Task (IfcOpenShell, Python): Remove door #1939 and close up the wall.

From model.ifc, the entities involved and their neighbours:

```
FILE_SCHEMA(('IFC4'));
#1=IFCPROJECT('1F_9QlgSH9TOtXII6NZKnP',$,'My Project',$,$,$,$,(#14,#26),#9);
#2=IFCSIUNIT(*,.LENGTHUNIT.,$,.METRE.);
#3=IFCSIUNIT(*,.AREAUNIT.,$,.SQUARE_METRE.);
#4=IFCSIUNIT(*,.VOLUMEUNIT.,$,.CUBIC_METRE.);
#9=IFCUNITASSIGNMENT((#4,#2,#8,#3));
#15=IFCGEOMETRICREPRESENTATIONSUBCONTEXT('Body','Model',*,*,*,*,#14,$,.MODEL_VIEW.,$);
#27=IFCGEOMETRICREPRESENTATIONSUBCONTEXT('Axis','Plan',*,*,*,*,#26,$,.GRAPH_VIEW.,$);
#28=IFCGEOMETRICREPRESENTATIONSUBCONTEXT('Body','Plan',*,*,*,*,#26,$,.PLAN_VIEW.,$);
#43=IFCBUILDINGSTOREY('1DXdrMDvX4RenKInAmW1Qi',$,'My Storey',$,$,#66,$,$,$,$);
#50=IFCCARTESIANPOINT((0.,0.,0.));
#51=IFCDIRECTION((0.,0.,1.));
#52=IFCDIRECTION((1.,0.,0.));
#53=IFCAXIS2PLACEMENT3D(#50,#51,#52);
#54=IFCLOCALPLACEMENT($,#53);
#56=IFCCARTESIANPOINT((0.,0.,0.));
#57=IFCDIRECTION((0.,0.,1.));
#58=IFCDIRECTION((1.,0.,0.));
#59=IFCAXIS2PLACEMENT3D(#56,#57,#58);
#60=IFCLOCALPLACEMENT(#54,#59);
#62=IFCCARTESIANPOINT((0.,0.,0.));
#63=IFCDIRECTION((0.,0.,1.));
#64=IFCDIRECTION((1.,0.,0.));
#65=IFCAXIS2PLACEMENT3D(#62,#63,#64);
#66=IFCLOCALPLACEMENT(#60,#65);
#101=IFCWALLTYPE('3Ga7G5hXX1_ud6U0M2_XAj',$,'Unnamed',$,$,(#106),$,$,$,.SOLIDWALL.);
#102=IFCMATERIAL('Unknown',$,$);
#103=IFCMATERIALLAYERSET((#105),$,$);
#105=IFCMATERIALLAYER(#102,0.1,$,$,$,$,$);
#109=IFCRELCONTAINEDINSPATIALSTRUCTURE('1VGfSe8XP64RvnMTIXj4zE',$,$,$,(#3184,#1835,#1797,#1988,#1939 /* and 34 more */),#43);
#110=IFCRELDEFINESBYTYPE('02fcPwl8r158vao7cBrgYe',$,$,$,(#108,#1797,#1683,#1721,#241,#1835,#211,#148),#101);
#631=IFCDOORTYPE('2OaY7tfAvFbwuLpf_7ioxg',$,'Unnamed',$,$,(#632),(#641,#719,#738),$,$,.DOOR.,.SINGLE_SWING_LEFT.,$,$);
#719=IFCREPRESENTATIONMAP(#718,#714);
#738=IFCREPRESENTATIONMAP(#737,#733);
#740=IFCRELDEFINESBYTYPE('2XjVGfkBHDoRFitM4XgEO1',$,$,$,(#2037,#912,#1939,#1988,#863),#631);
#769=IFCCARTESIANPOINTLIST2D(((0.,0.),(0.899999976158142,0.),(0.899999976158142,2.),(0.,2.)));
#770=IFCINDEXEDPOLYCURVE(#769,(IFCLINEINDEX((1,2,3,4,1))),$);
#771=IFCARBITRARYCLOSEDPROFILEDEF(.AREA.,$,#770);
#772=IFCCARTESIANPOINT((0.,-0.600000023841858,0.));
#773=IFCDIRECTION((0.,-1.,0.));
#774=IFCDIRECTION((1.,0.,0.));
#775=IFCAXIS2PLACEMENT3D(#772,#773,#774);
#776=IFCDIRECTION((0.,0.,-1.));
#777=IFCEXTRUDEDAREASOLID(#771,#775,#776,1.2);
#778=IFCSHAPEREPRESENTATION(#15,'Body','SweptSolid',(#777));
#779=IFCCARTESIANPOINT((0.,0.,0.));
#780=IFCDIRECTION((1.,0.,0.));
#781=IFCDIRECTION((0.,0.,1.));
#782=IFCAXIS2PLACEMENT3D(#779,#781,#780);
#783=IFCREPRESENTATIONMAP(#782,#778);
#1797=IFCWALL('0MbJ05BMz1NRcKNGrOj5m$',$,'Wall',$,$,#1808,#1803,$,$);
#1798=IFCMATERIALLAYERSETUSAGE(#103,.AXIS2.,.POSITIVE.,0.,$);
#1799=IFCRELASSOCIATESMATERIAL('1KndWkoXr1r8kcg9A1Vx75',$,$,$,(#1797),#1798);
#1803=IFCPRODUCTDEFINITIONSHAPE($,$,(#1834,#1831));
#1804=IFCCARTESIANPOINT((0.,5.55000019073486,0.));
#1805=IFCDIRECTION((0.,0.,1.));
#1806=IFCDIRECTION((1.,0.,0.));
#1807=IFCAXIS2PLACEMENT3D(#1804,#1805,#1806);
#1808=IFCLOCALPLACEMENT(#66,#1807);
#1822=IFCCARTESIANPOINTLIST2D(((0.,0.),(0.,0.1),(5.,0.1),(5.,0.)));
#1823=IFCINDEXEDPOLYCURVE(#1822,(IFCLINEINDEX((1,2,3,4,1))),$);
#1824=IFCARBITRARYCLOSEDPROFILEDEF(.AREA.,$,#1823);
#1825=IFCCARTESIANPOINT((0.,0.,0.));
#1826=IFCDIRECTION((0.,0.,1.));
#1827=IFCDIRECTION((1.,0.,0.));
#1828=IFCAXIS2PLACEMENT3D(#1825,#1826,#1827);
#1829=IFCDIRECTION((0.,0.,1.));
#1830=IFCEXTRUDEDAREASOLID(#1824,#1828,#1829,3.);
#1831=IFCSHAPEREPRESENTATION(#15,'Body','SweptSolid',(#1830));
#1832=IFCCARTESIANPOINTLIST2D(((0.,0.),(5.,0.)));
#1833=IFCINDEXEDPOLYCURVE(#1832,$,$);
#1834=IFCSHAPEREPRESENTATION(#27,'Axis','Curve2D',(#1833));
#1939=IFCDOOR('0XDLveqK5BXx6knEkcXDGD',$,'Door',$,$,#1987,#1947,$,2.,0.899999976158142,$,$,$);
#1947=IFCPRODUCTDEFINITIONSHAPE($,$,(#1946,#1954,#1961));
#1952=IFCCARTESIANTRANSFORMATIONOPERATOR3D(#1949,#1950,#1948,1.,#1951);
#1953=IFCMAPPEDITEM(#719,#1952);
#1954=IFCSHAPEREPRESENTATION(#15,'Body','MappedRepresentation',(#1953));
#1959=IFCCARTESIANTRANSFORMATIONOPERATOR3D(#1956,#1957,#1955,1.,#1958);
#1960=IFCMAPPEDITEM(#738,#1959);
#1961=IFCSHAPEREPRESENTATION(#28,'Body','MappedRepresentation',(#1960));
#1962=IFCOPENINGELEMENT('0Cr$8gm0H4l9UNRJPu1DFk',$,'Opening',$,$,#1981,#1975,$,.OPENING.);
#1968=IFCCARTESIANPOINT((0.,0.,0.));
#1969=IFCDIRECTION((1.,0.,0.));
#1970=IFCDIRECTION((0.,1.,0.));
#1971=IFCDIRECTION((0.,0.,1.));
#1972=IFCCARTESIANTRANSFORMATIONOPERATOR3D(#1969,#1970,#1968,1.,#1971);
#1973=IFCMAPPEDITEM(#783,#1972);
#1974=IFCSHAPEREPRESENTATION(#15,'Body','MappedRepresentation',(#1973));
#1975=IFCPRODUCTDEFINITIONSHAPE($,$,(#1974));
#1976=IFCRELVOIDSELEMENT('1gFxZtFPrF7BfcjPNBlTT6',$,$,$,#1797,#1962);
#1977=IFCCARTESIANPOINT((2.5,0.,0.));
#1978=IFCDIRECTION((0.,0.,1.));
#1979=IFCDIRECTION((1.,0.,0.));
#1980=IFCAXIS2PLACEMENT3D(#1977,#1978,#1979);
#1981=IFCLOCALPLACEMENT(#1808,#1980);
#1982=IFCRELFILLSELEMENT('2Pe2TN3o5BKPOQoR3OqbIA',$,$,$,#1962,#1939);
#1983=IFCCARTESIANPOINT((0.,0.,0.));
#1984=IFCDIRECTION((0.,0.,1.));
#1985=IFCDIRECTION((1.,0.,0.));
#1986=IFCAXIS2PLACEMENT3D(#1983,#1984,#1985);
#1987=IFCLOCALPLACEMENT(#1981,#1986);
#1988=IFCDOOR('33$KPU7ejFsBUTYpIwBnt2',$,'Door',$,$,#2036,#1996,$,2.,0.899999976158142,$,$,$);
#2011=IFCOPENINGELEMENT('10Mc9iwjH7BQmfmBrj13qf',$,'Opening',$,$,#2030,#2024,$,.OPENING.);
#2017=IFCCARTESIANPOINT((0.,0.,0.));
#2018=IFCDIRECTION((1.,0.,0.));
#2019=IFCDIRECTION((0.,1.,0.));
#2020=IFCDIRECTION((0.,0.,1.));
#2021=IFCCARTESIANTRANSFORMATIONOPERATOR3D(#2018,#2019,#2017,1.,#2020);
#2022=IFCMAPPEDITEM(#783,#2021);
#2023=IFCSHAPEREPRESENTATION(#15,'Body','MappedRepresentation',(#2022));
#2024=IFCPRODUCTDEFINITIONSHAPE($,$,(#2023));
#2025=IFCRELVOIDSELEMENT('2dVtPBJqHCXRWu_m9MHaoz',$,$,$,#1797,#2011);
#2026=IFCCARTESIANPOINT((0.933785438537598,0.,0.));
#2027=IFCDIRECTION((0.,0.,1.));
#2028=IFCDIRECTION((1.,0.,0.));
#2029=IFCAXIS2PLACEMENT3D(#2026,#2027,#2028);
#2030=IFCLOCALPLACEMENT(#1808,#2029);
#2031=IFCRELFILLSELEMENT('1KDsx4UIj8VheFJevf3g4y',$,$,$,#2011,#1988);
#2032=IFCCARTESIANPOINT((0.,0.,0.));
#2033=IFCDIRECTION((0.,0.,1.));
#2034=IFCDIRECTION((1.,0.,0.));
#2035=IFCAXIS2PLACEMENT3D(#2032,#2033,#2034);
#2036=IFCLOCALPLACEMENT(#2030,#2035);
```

```python
import ifcopenshell
import ifcopenshell.api.feature
import ifcopenshell.api.root
import ifcopenshell.geom
import ifcopenshell.util.shape

model = ifcopenshell.open("model.ifc")
settings = ifcopenshell.geom.settings()


def volume(element):
    """Net volume in cubic metres, openings subtracted."""
    shape = ifcopenshell.geom.create_shape(settings, element)
    return ifcopenshell.util.shape.get_volume(shape.geometry)


door = model.by_guid("0XDLveqK5BXx6knEkcXDGD")
opening = door.FillsVoids[0].RelatingOpeningElement
wall = opening.VoidsElements[0].RelatingBuildingElement
before = volume(wall)

ifcopenshell.api.root.remove_product(model, product=door)
ifcopenshell.api.feature.remove_feature(model, feature=opening)

after = volume(wall)

print(f"wall volume {before:.3f} -> {after:.3f} m3")

model.write("model_rev.ifc")
```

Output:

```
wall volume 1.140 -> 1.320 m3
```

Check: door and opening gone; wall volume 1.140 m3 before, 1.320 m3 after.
